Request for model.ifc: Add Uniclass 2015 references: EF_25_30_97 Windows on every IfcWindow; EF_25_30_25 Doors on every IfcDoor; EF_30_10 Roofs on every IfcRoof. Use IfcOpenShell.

First a look at what the model holds.

```python
import ifcopenshell

model = ifcopenshell.open("model.ifc")
print(model.schema)
print("classifications:", [c.Name for c in model.by_type("IfcClassification")])
for ifc_class in ("IfcDoor", "IfcRoof", "IfcStair", "IfcWall", "IfcWindow"):
    print(ifc_class, len(model.by_type(ifc_class)))
```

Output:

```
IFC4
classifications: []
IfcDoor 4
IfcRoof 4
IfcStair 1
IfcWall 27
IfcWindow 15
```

```python
import ifcopenshell
import ifcopenshell.api.classification

model = ifcopenshell.open("model.ifc")

system = ifcopenshell.api.classification.add_classification(model, classification="Uniclass 2015")

codes = {
    "IfcWindow": ("EF_25_30_97", "Windows"),
    "IfcDoor": ("EF_25_30_25", "Doors"),
    "IfcRoof": ("EF_30_10", "Roofs"),
}
for ifc_class, (code, name) in codes.items():
    products = model.by_type(ifc_class)
    ifcopenshell.api.classification.add_reference(
        model, products=products, classification=system, identification=code, name=name
    )
    print(code, len(products))

model.write("model-out.ifc")
```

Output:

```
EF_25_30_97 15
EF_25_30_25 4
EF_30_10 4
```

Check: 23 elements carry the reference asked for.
